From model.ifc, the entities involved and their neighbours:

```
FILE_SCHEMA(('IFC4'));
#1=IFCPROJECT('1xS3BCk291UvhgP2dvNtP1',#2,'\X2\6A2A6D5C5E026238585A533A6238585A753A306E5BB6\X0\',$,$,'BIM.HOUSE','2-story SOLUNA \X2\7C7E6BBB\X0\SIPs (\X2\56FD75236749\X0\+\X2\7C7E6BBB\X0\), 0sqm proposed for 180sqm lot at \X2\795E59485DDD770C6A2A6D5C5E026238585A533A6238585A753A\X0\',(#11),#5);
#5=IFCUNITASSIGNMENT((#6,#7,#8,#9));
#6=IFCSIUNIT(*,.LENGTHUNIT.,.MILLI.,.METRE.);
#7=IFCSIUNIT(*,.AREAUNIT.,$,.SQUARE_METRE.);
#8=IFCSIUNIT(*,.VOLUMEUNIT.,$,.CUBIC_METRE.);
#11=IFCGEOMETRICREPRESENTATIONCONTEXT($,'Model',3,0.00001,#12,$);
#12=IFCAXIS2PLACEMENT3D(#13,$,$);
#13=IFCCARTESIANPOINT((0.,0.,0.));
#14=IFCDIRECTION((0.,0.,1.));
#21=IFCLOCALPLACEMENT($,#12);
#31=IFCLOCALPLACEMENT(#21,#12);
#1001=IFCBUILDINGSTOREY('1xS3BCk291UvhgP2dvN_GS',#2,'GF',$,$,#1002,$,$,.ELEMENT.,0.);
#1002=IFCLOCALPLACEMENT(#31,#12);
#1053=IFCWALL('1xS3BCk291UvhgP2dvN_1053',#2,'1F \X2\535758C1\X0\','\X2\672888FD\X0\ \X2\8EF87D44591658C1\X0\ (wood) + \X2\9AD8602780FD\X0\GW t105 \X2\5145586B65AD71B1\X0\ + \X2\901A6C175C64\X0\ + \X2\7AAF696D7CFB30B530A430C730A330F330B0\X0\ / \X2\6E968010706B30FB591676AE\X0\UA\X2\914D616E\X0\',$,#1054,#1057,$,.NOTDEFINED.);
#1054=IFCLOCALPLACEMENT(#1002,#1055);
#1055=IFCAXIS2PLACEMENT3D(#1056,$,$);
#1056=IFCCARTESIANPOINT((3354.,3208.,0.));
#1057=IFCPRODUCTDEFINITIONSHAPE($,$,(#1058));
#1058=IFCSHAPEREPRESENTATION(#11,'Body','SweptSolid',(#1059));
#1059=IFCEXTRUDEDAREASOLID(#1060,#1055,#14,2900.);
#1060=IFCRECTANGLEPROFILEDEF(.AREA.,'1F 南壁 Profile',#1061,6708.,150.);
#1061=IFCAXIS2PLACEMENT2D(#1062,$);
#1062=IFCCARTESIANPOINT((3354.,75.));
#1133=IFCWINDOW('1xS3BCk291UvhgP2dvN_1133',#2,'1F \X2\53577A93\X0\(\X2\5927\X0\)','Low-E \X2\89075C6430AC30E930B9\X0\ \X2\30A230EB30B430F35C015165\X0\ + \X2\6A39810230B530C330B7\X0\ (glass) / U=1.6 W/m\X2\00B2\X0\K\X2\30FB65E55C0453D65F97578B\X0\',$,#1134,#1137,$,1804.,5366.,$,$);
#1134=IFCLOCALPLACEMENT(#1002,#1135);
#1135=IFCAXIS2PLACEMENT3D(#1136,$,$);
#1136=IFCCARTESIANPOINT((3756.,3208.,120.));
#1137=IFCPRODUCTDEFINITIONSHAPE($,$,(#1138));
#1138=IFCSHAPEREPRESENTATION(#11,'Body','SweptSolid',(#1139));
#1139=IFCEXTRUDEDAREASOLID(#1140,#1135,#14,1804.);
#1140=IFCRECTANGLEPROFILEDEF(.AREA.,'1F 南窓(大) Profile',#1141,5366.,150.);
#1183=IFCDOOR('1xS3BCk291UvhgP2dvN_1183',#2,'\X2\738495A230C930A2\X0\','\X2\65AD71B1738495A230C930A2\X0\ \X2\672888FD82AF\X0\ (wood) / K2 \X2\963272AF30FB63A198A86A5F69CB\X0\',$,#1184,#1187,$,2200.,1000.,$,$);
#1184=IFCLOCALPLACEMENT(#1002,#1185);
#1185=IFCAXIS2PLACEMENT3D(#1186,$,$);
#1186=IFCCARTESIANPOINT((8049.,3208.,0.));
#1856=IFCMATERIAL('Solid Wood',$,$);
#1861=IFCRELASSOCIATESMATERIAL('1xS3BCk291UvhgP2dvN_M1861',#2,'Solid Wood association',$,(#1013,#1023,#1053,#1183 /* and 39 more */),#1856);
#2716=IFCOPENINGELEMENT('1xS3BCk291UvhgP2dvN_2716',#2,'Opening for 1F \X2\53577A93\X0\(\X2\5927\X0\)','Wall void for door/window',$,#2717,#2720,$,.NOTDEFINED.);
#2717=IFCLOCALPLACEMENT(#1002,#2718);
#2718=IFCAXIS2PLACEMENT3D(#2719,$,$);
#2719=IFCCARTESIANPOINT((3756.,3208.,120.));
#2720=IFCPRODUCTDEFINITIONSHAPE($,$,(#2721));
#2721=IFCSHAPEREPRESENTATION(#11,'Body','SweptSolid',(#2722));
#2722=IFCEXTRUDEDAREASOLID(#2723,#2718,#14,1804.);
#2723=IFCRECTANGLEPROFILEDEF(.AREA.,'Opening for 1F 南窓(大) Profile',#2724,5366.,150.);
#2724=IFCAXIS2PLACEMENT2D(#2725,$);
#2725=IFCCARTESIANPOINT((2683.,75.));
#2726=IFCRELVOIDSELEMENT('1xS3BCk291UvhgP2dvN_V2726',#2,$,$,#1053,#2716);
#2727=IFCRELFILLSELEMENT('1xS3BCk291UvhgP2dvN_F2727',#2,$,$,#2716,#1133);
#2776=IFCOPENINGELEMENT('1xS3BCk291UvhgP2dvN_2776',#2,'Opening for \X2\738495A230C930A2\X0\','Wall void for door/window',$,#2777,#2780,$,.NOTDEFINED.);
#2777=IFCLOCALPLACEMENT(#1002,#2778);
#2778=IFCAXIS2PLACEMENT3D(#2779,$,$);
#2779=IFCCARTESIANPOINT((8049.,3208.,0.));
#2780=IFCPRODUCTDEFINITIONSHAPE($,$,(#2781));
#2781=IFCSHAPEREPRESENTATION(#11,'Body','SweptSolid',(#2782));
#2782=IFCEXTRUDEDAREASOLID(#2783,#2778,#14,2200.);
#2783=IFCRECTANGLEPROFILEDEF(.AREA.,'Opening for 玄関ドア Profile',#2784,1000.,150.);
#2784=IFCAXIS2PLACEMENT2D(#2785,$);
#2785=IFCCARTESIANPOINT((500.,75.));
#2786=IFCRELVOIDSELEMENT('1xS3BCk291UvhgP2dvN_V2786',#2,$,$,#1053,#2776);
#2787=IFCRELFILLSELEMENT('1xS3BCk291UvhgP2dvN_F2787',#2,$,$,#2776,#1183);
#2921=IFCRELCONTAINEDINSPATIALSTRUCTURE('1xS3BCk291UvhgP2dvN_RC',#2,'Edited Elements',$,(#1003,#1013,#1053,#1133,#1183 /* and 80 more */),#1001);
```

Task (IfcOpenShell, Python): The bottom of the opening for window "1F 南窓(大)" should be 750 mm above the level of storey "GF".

```python
import numpy as np
import ifcopenshell
import ifcopenshell.api.geometry
import ifcopenshell.geom
import ifcopenshell.util.element
import ifcopenshell.util.placement
import ifcopenshell.util.shape
import ifcopenshell.util.unit

model = ifcopenshell.open("model.ifc")
unit_scale = ifcopenshell.util.unit.calculate_unit_scale(model)

window = model.by_guid("1xS3BCk291UvhgP2dvN_1133")
opening = window.FillsVoids[0].RelatingOpeningElement
storey = ifcopenshell.util.element.get_container(window, ifc_class="IfcBuildingStorey")
level = ifcopenshell.util.placement.get_local_placement(storey.ObjectPlacement)[2, 3]

# The opening's origin need not be at the sill, so measure its lowest point.
shape = ifcopenshell.geom.create_shape(ifcopenshell.geom.settings(), opening)
bottom = ifcopenshell.util.shape.get_shape_bottom_elevation(shape, shape.geometry) / unit_scale
dz = level + 750.0 - bottom

shift = np.array([0.0, 0.0, dz])
# The window is not placed relative to its opening, so move both.
for product in (opening, window):
    matrix = ifcopenshell.util.placement.get_local_placement(product.ObjectPlacement)
    matrix[:3, 3] += shift
    ifcopenshell.api.geometry.edit_object_placement(model, product=product, matrix=matrix, is_si=False)

print(f"moved by {dz * unit_scale:+.3f} m")

model.write("model_updated.ifc")
```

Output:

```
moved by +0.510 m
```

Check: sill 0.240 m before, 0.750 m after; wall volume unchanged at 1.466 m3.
